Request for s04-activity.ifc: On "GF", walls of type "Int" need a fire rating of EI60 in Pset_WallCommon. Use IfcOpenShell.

First a look at what the model holds.

```python
import ifcopenshell
import ifcopenshell.util.element

model = ifcopenshell.open("s04-activity.ifc")
print(model.schema)
storey = next(s for s in model.by_type("IfcBuildingStorey") if s.Name == "GF")
walls = [e for e in ifcopenshell.util.element.get_decomposition(storey) if e.is_a("IfcWall")]
seen = {}
for e in walls:
    element_type = ifcopenshell.util.element.get_type(e)
    key = (element_type.Name if element_type != e and element_type else None, ifcopenshell.util.element.get_pset(e, "Pset_WallCommon", "FireRating"))
    seen[key] = seen.get(key, 0) + 1
for (name, value), count in sorted(seen.items(), key=str):
    print(count, "x", name, "|", value)
```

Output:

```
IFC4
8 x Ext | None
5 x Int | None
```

```python
import ifcopenshell
import ifcopenshell.api.pset
import ifcopenshell.util.element

model = ifcopenshell.open("s04-activity.ifc")

storey = next(s for s in model.by_type("IfcBuildingStorey") if s.Name == "GF")
walls = [e for e in ifcopenshell.util.element.get_decomposition(storey) if e.is_a("IfcWall")]

count = 0
for e in walls:
    element_type = ifcopenshell.util.element.get_type(e)
    if element_type in (None, e) or element_type.Name != "Int":
        continue
    # add_pset returns the element's existing set when there is one.
    pset = ifcopenshell.api.pset.add_pset(model, product=e, name="Pset_WallCommon")
    ifcopenshell.api.pset.edit_pset(model, pset=pset, properties={"FireRating": "EI60"})
    count += 1

print(count, "walls updated")

model.write("s04-activity_updated.ifc")
```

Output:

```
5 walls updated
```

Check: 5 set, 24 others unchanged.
